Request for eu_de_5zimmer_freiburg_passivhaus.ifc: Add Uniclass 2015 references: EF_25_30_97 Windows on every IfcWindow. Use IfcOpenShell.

First a look at what the model holds.

```python
import ifcopenshell

model = ifcopenshell.open("eu_de_5zimmer_freiburg_passivhaus.ifc")
print(model.schema)
print("classifications:", [c.Name for c in model.by_type("IfcClassification")])
for ifc_class in ("IfcDoor", "IfcRoof", "IfcStair", "IfcWall", "IfcWindow"):
    print(ifc_class, len(model.by_type(ifc_class)))
```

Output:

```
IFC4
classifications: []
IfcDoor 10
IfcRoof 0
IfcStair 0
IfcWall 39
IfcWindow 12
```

```python
import ifcopenshell
import ifcopenshell.api.classification

model = ifcopenshell.open("eu_de_5zimmer_freiburg_passivhaus.ifc")

system = ifcopenshell.api.classification.add_classification(model, classification="Uniclass 2015")

codes = {
    "IfcWindow": ("EF_25_30_97", "Windows"),
}
for ifc_class, (code, name) in codes.items():
    products = model.by_type(ifc_class)
    ifcopenshell.api.classification.add_reference(
        model, products=products, classification=system, identification=code, name=name
    )
    print(code, len(products))

model.write("eu_de_5zimmer_freiburg_passivhaus_updated.ifc")
```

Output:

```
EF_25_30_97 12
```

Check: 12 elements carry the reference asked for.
